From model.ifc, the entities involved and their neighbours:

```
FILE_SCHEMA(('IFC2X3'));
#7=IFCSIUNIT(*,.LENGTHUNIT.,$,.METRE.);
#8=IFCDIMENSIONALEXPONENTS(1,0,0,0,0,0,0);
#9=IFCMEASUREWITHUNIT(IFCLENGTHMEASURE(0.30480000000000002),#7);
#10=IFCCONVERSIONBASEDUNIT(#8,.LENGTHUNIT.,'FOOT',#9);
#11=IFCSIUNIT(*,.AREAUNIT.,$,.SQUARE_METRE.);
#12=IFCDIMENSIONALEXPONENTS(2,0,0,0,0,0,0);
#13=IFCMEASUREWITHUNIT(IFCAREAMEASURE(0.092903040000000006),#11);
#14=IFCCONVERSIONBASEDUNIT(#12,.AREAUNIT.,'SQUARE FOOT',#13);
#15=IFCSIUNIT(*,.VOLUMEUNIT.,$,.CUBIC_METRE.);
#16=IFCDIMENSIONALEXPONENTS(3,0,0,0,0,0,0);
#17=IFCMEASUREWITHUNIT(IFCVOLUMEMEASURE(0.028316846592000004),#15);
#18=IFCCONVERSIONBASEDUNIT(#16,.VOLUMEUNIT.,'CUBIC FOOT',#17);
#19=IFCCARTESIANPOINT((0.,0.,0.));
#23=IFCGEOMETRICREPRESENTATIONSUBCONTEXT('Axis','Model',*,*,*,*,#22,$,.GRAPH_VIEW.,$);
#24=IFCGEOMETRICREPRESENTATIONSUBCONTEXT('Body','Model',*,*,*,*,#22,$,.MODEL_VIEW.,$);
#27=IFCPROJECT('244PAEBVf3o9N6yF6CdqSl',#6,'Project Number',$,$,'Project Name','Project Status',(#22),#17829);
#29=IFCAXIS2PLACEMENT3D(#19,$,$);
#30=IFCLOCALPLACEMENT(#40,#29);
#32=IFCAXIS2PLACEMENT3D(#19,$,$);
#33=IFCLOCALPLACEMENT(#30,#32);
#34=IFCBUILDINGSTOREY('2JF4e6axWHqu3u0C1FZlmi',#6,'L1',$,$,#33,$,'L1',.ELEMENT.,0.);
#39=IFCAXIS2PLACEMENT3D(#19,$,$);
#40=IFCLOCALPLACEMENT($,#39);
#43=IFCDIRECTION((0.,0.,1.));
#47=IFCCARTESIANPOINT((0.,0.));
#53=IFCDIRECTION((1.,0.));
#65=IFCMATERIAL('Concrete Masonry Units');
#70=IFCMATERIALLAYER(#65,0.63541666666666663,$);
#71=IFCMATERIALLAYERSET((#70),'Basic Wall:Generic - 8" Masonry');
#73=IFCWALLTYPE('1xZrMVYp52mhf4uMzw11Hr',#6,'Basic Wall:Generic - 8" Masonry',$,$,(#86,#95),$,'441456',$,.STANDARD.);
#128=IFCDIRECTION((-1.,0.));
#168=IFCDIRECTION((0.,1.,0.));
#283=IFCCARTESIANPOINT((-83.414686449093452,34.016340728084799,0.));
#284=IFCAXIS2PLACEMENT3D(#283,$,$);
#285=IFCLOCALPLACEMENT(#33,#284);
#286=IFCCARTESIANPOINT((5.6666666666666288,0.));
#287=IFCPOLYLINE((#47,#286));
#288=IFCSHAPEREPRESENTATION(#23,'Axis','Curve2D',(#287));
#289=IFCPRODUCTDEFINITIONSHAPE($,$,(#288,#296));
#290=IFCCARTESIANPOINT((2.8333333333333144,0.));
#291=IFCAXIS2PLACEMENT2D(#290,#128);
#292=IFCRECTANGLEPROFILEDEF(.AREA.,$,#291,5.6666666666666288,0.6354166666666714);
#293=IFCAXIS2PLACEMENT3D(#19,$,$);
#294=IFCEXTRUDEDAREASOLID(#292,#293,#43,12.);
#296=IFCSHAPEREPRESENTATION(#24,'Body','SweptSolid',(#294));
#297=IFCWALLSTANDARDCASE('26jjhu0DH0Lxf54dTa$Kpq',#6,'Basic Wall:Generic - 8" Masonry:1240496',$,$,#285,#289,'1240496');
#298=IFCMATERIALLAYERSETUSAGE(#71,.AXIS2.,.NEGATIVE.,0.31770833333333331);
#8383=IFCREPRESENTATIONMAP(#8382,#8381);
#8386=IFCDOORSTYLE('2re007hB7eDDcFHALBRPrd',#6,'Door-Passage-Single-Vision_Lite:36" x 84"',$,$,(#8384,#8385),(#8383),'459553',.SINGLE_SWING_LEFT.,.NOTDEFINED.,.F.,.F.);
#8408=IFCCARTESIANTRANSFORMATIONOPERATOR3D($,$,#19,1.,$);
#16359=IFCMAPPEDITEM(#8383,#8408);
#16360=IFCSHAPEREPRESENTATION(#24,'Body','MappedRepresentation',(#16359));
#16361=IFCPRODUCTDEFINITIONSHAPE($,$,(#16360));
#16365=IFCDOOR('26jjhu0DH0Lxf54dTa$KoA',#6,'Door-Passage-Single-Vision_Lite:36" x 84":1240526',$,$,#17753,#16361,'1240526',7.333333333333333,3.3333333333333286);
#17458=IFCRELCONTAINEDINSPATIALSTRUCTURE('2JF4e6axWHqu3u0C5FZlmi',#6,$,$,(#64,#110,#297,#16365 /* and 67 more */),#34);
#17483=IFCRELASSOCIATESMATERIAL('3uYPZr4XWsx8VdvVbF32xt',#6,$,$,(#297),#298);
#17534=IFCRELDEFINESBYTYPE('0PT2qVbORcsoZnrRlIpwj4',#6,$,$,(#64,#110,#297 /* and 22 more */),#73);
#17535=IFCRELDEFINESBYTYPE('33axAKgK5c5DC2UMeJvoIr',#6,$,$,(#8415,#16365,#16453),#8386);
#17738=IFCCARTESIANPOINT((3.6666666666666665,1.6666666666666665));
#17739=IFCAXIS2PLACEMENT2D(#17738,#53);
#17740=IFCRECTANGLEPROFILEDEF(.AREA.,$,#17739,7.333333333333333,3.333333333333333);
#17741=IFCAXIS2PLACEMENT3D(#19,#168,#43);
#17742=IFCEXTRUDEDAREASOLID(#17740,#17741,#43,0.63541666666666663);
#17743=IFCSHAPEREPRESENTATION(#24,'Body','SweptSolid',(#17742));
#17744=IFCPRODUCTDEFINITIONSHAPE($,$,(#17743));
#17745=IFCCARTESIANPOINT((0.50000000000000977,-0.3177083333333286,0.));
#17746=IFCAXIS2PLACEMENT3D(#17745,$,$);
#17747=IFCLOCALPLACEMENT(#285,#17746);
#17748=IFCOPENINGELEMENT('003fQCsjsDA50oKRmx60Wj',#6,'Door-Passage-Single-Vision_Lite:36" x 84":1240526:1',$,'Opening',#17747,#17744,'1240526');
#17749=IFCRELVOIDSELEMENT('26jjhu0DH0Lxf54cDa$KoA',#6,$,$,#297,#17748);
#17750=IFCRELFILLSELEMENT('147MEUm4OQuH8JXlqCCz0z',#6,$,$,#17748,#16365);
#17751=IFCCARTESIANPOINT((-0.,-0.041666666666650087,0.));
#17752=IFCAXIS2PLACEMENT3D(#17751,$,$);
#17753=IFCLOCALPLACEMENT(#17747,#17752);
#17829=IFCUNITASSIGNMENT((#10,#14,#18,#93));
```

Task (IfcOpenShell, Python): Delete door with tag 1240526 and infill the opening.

```python
import ifcopenshell
import ifcopenshell.api.feature
import ifcopenshell.api.root
import ifcopenshell.geom
import ifcopenshell.util.shape

model = ifcopenshell.open("model.ifc")
settings = ifcopenshell.geom.settings()


def volume(element):
    """Net volume in cubic metres, openings subtracted."""
    shape = ifcopenshell.geom.create_shape(settings, element)
    return ifcopenshell.util.shape.get_volume(shape.geometry)


door = model.by_id(16365)
opening = door.FillsVoids[0].RelatingOpeningElement
wall = opening.VoidsElements[0].RelatingBuildingElement
before = volume(wall)

ifcopenshell.api.root.remove_product(model, product=door)
ifcopenshell.api.feature.remove_feature(model, feature=opening)

after = volume(wall)

print(f"wall volume {before:.3f} -> {after:.3f} m3")

model.write("model-out.ifc")
```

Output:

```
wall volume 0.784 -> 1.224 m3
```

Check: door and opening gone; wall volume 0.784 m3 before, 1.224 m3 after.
